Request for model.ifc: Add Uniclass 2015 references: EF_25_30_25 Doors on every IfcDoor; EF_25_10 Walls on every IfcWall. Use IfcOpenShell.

First a look at what the model holds.

```python
import ifcopenshell

model = ifcopenshell.open("model.ifc")
print(model.schema)
print("classifications:", [c.Name for c in model.by_type("IfcClassification")])
for ifc_class in ("IfcDoor", "IfcRoof", "IfcStair", "IfcWall", "IfcWindow"):
    print(ifc_class, len(model.by_type(ifc_class)))
```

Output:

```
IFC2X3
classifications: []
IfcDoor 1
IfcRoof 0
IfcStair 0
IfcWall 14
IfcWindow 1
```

```python
import ifcopenshell
import ifcopenshell.api.classification

model = ifcopenshell.open("model.ifc")

# IFC2X3 requires Source and Edition and has no link from the project to the system.
system = model.create_entity("IfcClassification", Source="NBS", Edition="2015", Name="Uniclass 2015")

codes = {
    "IfcDoor": ("EF_25_30_25", "Doors"),
    "IfcWall": ("EF_25_10", "Walls"),
}
for ifc_class, (code, name) in codes.items():
    products = model.by_type(ifc_class)
    ifcopenshell.api.classification.add_reference(
        model, products=products, classification=system, identification=code, name=name
    )
    print(code, len(products))

model.write("model_rev.ifc")
```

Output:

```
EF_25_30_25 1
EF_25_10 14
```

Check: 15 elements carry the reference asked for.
